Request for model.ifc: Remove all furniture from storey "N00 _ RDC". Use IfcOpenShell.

First a look at what the model holds.

```python
import ifcopenshell
import ifcopenshell.util.element

model = ifcopenshell.open("model.ifc")
print(model.schema)
storey = next(s for s in model.by_type("IfcBuildingStorey") if s.Name == "N00 _ RDC")
furniture = [e for e in ifcopenshell.util.element.get_decomposition(storey) if e.is_a("IfcFurnishingElement")]
seen = {}
for e in furniture:
    element_type = ifcopenshell.util.element.get_type(e)
    name = element_type.Name if element_type not in (None, e) else None
    seen[name] = seen.get(name, 0) + 1
for name, count in sorted(seen.items(), key=str):
    print(count, "x", name)
```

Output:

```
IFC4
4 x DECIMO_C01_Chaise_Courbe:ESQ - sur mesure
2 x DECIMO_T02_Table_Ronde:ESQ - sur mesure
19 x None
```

```python
import ifcopenshell
import ifcopenshell.api.root
import ifcopenshell.util.element

model = ifcopenshell.open("model.ifc")

storey = next(s for s in model.by_type("IfcBuildingStorey") if s.Name == "N00 _ RDC")
furniture = [e for e in ifcopenshell.util.element.get_decomposition(storey) if e.is_a("IfcFurnishingElement")]

for e in furniture:
    ifcopenshell.api.root.remove_product(model, product=e)
print(len(furniture), "removed")

model.write("model-out.ifc")
```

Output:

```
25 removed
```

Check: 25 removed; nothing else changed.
